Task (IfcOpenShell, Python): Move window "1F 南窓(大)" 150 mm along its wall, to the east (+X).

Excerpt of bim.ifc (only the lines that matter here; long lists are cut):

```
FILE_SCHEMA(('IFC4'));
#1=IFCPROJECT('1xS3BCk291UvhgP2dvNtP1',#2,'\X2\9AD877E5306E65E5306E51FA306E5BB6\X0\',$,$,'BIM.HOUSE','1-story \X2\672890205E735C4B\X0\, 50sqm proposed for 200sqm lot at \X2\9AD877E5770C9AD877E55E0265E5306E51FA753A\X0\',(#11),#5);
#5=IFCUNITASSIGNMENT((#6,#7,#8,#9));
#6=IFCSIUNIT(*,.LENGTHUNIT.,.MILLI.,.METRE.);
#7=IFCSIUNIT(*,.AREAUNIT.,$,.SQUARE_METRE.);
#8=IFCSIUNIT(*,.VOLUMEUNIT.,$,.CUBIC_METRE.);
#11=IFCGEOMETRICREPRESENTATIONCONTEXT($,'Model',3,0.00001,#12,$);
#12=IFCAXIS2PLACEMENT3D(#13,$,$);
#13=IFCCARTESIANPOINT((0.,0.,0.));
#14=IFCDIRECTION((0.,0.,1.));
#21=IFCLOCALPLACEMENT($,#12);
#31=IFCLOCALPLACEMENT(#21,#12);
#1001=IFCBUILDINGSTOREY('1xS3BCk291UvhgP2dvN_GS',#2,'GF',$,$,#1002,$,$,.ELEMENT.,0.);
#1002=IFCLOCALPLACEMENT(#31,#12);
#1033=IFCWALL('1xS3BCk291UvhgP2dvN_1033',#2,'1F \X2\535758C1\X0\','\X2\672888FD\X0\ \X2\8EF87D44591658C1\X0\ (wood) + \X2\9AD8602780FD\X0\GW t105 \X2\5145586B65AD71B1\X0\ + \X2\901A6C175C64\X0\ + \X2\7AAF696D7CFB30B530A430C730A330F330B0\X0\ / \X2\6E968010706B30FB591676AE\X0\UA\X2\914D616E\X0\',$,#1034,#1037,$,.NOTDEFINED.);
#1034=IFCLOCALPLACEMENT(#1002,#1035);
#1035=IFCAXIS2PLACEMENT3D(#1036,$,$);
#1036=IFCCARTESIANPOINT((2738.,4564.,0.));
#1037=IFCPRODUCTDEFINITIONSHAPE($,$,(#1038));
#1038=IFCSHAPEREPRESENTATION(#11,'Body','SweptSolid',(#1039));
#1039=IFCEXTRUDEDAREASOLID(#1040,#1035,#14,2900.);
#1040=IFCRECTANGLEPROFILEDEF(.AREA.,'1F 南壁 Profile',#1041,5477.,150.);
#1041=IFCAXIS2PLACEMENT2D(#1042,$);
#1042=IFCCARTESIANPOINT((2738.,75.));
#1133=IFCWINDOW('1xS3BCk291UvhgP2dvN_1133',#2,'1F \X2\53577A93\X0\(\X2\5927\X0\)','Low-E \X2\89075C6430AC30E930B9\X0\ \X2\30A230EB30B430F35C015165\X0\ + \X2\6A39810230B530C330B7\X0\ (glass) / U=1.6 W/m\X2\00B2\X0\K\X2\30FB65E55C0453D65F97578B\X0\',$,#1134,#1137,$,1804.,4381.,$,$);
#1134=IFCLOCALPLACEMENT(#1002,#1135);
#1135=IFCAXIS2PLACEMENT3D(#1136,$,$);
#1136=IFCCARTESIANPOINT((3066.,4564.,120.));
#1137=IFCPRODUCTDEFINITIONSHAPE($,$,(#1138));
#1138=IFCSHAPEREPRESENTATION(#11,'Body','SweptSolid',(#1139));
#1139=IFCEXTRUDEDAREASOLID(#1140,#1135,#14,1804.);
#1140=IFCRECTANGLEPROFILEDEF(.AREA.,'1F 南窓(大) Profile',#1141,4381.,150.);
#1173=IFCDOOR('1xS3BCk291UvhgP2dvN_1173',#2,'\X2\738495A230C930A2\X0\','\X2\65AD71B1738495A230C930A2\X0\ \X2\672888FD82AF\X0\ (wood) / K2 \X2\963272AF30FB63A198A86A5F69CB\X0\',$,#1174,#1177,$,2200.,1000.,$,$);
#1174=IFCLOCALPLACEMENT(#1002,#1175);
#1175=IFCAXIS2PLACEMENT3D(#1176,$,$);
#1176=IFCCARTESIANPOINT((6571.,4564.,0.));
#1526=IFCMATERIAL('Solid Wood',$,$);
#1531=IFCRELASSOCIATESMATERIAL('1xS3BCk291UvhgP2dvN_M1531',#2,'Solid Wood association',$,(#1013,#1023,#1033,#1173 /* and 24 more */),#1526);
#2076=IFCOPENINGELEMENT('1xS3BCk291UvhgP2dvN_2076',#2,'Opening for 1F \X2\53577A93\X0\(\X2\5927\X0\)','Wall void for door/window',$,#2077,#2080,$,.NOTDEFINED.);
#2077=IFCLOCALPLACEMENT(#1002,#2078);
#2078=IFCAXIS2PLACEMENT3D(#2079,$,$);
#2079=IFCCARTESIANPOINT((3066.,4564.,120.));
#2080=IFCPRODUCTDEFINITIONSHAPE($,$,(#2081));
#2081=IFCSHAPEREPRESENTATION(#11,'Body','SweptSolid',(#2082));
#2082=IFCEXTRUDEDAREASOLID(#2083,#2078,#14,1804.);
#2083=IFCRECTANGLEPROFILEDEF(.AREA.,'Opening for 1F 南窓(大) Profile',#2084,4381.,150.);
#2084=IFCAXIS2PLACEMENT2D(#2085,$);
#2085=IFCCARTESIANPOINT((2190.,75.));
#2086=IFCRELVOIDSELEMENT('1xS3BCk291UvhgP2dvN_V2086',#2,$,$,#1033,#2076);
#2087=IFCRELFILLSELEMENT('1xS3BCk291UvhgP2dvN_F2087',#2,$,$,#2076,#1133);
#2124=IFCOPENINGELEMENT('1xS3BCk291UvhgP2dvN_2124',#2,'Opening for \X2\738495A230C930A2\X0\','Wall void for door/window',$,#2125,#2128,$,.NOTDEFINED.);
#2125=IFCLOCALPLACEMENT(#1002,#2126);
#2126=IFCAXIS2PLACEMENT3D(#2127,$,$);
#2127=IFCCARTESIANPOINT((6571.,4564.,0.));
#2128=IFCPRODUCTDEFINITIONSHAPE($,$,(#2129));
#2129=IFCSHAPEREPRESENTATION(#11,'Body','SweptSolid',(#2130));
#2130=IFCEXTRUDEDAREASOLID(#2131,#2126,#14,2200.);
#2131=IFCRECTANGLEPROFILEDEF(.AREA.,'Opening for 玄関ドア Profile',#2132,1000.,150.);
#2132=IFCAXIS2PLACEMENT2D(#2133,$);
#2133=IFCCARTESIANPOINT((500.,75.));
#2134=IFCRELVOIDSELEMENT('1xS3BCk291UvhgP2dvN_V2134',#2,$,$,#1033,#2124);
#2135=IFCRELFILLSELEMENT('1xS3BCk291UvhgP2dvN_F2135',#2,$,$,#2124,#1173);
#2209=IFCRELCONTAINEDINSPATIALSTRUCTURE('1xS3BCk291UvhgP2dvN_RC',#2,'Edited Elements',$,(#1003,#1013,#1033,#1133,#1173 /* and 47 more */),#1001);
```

```python
import ifcopenshell
import ifcopenshell.api.geometry
import ifcopenshell.util.placement
import ifcopenshell.util.unit

model = ifcopenshell.open("bim.ifc")
unit_scale = ifcopenshell.util.unit.calculate_unit_scale(model)

window = model.by_guid("1xS3BCk291UvhgP2dvN_1133")
opening = window.FillsVoids[0].RelatingOpeningElement
wall = opening.VoidsElements[0].RelatingBuildingElement

wall_matrix = ifcopenshell.util.placement.get_local_placement(wall.ObjectPlacement)
shift = wall_matrix[:3, 0] * 0.15 / unit_scale
before = ifcopenshell.util.placement.get_local_placement(window.ObjectPlacement)[:3, 3].copy()

# The window is not placed relative to its opening, so move both.
for product in (opening, window):
    matrix = ifcopenshell.util.placement.get_local_placement(product.ObjectPlacement)
    matrix[:3, 3] += shift
    ifcopenshell.api.geometry.edit_object_placement(model, product=product, matrix=matrix, is_si=False)

after = ifcopenshell.util.placement.get_local_placement(window.ObjectPlacement)[:3, 3]
print("window moved by", (after - before).round(3) + 0.0)

model.write("bim_v2.ifc")
```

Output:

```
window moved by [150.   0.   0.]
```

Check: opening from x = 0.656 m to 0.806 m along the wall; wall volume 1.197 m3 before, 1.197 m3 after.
